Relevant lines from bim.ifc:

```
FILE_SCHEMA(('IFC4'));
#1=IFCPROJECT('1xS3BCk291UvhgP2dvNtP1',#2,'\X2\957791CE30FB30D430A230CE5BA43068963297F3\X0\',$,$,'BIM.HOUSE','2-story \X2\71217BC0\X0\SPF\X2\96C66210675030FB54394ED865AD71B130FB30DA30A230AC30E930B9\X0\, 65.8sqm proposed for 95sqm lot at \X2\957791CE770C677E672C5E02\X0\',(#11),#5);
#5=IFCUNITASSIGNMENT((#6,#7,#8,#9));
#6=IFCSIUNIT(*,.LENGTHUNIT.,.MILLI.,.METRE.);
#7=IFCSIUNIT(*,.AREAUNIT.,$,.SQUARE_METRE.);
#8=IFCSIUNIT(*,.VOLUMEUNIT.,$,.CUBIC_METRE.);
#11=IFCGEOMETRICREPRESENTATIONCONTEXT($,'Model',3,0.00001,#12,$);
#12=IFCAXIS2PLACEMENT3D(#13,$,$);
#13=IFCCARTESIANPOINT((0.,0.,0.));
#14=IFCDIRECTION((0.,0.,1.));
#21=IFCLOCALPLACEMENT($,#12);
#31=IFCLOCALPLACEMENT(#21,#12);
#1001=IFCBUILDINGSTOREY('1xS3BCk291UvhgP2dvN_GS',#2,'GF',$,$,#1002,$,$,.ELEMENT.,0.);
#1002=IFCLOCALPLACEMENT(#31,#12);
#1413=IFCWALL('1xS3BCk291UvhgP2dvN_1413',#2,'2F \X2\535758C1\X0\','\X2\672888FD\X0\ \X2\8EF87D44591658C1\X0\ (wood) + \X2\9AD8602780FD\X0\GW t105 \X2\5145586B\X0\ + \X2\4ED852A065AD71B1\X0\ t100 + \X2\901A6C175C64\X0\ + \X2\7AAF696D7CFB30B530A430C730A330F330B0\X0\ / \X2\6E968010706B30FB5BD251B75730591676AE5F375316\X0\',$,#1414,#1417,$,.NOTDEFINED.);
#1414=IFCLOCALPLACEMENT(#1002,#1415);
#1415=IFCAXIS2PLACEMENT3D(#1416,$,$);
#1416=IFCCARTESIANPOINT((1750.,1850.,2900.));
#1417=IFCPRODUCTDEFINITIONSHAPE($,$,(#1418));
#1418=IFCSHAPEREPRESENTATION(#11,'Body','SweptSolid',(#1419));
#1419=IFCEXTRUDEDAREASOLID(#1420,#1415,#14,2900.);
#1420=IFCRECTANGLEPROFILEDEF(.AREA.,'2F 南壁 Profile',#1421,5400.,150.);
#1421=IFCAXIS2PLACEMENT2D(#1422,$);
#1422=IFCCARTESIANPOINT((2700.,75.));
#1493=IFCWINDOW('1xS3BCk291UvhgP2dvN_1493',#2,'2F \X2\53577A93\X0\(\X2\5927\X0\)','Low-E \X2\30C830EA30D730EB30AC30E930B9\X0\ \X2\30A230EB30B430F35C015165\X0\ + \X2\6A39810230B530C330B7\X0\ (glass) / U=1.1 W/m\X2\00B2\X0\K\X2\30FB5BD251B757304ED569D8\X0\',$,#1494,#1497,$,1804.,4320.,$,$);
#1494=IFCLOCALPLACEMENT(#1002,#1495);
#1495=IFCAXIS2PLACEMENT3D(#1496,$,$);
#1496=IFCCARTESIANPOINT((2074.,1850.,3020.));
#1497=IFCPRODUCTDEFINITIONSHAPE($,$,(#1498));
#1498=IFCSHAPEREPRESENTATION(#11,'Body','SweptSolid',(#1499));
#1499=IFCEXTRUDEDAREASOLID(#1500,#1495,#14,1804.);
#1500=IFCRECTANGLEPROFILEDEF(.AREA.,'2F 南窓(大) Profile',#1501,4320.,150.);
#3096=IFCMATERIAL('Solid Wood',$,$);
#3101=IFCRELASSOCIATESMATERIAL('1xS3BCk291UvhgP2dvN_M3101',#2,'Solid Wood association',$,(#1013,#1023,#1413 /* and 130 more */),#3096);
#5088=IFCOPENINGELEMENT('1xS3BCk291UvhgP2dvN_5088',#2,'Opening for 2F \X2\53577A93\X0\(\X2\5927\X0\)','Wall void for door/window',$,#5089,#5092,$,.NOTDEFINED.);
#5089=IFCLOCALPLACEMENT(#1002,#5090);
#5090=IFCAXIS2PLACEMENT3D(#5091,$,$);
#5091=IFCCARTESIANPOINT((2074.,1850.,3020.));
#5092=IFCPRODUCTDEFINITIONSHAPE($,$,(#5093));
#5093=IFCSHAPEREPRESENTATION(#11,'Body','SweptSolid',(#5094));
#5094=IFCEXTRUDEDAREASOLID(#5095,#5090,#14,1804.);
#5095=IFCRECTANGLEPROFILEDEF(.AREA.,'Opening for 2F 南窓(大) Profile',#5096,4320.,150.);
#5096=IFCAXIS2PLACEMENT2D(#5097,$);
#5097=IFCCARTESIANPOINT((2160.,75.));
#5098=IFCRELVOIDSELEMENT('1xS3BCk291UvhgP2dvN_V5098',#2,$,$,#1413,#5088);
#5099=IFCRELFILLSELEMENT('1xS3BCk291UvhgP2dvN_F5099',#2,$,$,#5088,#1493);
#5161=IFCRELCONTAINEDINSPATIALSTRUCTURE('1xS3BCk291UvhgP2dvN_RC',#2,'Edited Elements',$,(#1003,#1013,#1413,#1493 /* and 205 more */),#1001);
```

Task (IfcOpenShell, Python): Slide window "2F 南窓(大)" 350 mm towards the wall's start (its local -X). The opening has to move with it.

```python
import ifcopenshell
import ifcopenshell.api.geometry
import ifcopenshell.util.placement

model = ifcopenshell.open("bim.ifc")

window = model.by_guid("1xS3BCk291UvhgP2dvN_1493")
opening = window.FillsVoids[0].RelatingOpeningElement
wall = opening.VoidsElements[0].RelatingBuildingElement

wall_matrix = ifcopenshell.util.placement.get_local_placement(wall.ObjectPlacement)
shift = wall_matrix[:3, 0] * -350.0
before = ifcopenshell.util.placement.get_local_placement(window.ObjectPlacement)[:3, 3].copy()

# The window is not placed relative to its opening, so move both.
for product in (opening, window):
    matrix = ifcopenshell.util.placement.get_local_placement(product.ObjectPlacement)
    matrix[:3, 3] += shift
    ifcopenshell.api.geometry.edit_object_placement(model, product=product, matrix=matrix, is_si=False)

after = ifcopenshell.util.placement.get_local_placement(window.ObjectPlacement)[:3, 3]
print("window moved by", (after - before).round(3) + 0.0)

model.write("bim_updated.ifc")
```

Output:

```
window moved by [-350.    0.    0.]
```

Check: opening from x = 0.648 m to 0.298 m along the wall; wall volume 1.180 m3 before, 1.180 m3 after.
